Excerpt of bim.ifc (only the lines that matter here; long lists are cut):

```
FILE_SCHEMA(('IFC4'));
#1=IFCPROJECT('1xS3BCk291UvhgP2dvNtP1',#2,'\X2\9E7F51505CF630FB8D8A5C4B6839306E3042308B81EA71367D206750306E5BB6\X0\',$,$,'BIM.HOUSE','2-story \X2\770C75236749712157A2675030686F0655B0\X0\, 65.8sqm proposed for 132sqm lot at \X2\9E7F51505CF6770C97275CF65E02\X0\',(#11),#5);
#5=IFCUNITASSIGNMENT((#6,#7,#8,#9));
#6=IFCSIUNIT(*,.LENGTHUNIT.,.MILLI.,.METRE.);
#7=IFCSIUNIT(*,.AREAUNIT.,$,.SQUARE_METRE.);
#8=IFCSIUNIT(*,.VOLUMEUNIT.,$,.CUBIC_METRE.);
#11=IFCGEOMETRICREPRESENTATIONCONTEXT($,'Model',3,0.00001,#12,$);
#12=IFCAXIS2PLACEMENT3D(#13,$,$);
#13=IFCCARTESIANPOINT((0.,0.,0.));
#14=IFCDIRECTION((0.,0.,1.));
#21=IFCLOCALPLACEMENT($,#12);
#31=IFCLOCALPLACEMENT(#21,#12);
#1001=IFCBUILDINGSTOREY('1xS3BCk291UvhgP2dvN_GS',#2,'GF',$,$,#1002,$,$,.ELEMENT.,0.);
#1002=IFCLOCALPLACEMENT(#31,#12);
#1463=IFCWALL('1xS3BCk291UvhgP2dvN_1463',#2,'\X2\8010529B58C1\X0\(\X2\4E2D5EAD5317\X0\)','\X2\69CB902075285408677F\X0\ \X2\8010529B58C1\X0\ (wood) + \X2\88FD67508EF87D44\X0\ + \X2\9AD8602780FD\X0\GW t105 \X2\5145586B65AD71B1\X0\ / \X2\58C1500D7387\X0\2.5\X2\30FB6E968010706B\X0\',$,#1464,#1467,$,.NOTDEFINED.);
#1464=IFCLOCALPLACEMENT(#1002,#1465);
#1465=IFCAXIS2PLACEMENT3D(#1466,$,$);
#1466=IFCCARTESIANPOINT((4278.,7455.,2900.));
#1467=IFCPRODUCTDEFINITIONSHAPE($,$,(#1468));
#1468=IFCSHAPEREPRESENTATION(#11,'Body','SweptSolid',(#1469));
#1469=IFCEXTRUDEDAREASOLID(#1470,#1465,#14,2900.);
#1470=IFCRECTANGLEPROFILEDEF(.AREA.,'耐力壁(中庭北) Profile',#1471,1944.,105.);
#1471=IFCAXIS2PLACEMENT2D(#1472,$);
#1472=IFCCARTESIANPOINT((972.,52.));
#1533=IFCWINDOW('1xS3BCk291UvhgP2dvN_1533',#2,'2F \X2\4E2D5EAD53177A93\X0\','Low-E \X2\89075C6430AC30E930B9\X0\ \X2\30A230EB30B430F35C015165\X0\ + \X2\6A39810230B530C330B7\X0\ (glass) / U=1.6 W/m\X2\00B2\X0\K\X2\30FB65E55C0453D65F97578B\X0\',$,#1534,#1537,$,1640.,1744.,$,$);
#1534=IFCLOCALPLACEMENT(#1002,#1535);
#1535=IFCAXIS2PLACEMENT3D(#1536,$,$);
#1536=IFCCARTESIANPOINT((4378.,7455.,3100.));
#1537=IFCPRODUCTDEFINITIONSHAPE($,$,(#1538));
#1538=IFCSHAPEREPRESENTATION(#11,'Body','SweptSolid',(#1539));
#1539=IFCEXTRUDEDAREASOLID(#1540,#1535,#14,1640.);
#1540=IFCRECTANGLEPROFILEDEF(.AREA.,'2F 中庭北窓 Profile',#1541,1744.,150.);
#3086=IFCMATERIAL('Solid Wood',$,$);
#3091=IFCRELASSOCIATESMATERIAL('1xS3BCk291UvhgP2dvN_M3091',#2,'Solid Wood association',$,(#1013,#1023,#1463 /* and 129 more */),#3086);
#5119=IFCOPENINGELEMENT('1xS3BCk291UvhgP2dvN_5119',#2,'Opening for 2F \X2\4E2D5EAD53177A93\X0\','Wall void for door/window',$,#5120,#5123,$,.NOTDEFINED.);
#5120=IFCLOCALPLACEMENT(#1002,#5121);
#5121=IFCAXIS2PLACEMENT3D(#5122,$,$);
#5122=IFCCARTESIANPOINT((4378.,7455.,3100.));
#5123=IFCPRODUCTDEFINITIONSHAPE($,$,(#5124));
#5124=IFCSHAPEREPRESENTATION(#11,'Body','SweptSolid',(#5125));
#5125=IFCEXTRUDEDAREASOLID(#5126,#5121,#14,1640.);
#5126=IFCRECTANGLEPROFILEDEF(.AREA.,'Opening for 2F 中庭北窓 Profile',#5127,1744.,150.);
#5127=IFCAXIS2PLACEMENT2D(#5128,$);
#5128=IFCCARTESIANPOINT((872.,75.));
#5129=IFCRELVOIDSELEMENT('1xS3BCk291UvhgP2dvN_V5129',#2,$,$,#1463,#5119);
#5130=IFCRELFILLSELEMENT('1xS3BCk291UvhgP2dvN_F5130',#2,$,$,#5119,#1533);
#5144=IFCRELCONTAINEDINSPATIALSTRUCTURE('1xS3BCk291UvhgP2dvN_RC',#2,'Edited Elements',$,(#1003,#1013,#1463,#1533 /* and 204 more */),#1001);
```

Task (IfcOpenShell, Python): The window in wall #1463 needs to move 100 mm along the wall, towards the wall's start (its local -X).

```python
import ifcopenshell
import ifcopenshell.api.geometry
import ifcopenshell.util.placement
import ifcopenshell.util.unit

model = ifcopenshell.open("bim.ifc")
unit_scale = ifcopenshell.util.unit.calculate_unit_scale(model)

window = model.by_guid("1xS3BCk291UvhgP2dvN_1533")
opening = window.FillsVoids[0].RelatingOpeningElement
wall = opening.VoidsElements[0].RelatingBuildingElement

wall_matrix = ifcopenshell.util.placement.get_local_placement(wall.ObjectPlacement)
shift = wall_matrix[:3, 0] * -0.1 / unit_scale
before = ifcopenshell.util.placement.get_local_placement(window.ObjectPlacement)[:3, 3].copy()

# The window is not placed relative to its opening, so move both.
for product in (opening, window):
    matrix = ifcopenshell.util.placement.get_local_placement(product.ObjectPlacement)
    matrix[:3, 3] += shift
    ifcopenshell.api.geometry.edit_object_placement(model, product=product, matrix=matrix, is_si=False)

after = ifcopenshell.util.placement.get_local_placement(window.ObjectPlacement)[:3, 3]
print("window moved by", (after - before).round(3) + 0.0)

model.write("bim-out.ifc")
```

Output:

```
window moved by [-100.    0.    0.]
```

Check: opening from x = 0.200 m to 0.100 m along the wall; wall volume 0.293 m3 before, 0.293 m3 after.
